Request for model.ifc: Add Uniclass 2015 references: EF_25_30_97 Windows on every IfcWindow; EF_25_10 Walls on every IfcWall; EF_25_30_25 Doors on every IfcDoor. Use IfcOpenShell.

First a look at what the model holds.

```python
import ifcopenshell

model = ifcopenshell.open("model.ifc")
print(model.schema)
print("classifications:", [c.Name for c in model.by_type("IfcClassification")])
for ifc_class in ("IfcDoor", "IfcRoof", "IfcStair", "IfcWall", "IfcWindow"):
    print(ifc_class, len(model.by_type(ifc_class)))
```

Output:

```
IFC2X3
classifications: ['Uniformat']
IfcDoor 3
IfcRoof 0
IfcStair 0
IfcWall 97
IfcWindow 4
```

```python
import ifcopenshell
import ifcopenshell.api.classification

model = ifcopenshell.open("model.ifc")

# IFC2X3 requires Source and Edition and has no link from the project to the system.
system = model.create_entity("IfcClassification", Source="NBS", Edition="2015", Name="Uniclass 2015")

codes = {
    "IfcWindow": ("EF_25_30_97", "Windows"),
    "IfcWall": ("EF_25_10", "Walls"),
    "IfcDoor": ("EF_25_30_25", "Doors"),
}
for ifc_class, (code, name) in codes.items():
    products = model.by_type(ifc_class)
    ifcopenshell.api.classification.add_reference(
        model, products=products, classification=system, identification=code, name=name
    )
    print(code, len(products))

model.write("model_rev.ifc")
```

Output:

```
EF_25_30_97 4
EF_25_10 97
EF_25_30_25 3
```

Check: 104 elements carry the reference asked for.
